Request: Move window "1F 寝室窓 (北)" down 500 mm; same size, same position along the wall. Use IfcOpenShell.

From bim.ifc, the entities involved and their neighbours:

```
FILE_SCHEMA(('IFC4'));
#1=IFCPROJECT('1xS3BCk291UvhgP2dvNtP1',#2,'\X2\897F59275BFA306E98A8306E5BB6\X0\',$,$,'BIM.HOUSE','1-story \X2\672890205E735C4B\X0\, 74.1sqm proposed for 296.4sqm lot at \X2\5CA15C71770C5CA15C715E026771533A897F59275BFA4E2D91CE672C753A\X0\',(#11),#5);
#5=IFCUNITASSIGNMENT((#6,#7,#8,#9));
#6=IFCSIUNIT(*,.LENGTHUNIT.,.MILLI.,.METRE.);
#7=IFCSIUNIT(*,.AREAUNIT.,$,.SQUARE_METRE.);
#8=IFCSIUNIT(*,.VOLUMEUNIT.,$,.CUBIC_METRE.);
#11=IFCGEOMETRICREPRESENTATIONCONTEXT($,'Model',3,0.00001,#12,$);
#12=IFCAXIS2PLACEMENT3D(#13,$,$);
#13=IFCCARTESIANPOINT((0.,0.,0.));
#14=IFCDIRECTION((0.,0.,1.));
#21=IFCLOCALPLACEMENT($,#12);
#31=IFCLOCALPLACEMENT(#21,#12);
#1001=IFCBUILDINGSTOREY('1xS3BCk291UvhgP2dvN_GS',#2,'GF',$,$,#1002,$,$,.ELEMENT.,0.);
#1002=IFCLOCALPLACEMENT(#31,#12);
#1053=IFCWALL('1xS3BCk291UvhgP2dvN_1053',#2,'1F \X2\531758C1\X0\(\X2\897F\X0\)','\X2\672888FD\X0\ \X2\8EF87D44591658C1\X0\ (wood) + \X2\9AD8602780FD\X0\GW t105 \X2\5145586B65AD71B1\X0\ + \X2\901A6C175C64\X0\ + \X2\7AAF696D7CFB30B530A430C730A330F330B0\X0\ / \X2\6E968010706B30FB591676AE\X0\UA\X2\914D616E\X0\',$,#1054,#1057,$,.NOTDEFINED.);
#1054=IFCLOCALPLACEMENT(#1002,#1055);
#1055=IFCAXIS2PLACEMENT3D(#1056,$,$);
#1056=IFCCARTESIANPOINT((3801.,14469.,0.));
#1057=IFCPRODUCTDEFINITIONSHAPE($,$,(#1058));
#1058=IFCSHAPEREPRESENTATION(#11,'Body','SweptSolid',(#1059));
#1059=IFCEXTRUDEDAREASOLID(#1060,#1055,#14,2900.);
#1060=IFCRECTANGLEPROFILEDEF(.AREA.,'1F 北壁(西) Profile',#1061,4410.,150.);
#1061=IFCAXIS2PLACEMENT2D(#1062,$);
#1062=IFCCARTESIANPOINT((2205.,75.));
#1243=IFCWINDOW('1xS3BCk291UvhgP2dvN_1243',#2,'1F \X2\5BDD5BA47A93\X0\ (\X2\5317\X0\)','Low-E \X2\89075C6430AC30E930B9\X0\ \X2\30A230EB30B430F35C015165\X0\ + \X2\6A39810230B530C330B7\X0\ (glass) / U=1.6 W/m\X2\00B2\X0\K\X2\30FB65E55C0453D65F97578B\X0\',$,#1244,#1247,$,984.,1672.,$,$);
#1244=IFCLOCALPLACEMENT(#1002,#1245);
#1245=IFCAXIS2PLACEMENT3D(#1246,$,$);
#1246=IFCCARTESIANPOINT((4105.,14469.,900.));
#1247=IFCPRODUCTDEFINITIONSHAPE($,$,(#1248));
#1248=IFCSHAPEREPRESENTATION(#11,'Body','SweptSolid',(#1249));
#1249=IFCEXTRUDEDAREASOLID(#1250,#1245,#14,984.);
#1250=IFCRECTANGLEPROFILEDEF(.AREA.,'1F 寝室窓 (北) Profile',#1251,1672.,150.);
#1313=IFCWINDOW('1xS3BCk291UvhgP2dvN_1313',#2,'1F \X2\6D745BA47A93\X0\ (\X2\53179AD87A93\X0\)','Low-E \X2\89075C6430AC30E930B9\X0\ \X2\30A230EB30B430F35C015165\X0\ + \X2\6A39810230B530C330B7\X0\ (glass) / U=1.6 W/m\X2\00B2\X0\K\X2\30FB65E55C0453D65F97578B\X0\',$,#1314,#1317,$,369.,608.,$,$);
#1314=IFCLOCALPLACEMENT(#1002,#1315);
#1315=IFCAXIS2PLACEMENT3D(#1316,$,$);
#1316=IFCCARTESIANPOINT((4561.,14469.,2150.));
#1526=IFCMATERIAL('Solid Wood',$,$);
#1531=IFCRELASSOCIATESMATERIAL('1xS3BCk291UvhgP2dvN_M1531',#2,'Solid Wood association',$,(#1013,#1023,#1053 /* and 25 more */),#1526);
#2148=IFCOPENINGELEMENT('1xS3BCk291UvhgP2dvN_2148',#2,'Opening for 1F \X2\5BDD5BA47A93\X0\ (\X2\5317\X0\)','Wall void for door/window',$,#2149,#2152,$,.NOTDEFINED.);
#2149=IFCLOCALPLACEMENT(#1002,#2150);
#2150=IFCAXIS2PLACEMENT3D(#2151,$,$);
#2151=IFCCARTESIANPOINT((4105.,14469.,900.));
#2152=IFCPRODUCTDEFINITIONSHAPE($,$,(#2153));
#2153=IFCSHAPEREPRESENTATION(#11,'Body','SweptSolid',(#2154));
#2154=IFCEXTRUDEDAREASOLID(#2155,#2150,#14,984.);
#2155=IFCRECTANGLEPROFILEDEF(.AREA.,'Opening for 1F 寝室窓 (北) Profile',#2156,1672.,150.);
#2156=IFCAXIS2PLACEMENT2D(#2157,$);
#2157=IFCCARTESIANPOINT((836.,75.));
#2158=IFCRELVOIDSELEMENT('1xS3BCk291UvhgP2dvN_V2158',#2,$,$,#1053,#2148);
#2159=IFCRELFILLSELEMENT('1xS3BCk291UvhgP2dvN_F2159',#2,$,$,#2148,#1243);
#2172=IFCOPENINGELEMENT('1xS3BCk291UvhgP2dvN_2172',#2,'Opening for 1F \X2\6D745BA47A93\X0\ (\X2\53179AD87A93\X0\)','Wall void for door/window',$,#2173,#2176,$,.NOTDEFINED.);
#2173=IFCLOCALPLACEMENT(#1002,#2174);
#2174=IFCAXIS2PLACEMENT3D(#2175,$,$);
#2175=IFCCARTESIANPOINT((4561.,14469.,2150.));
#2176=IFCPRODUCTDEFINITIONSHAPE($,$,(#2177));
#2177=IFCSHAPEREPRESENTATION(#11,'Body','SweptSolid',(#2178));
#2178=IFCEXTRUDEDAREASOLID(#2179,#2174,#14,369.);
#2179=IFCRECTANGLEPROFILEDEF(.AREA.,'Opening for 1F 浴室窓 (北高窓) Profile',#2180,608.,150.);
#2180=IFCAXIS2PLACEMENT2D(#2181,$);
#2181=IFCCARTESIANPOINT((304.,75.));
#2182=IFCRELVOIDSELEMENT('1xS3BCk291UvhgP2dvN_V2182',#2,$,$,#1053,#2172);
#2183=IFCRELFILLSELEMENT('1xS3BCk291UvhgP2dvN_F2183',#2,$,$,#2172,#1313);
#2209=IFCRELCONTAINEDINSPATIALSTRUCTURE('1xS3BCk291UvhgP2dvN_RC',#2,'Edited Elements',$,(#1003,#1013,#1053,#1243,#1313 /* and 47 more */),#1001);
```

```python
import numpy as np
import ifcopenshell
import ifcopenshell.api.geometry
import ifcopenshell.util.placement
import ifcopenshell.util.unit

model = ifcopenshell.open("bim.ifc")
unit_scale = ifcopenshell.util.unit.calculate_unit_scale(model)

window = model.by_guid("1xS3BCk291UvhgP2dvN_1243")
opening = window.FillsVoids[0].RelatingOpeningElement
dz = -0.5 / unit_scale

shift = np.array([0.0, 0.0, dz])
# The window is not placed relative to its opening, so move both.
for product in (opening, window):
    matrix = ifcopenshell.util.placement.get_local_placement(product.ObjectPlacement)
    matrix[:3, 3] += shift
    ifcopenshell.api.geometry.edit_object_placement(model, product=product, matrix=matrix, is_si=False)

print(f"moved by {dz * unit_scale:+.3f} m")

model.write("bim-out.ifc")
```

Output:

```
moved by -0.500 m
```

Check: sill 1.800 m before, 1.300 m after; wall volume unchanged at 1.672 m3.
